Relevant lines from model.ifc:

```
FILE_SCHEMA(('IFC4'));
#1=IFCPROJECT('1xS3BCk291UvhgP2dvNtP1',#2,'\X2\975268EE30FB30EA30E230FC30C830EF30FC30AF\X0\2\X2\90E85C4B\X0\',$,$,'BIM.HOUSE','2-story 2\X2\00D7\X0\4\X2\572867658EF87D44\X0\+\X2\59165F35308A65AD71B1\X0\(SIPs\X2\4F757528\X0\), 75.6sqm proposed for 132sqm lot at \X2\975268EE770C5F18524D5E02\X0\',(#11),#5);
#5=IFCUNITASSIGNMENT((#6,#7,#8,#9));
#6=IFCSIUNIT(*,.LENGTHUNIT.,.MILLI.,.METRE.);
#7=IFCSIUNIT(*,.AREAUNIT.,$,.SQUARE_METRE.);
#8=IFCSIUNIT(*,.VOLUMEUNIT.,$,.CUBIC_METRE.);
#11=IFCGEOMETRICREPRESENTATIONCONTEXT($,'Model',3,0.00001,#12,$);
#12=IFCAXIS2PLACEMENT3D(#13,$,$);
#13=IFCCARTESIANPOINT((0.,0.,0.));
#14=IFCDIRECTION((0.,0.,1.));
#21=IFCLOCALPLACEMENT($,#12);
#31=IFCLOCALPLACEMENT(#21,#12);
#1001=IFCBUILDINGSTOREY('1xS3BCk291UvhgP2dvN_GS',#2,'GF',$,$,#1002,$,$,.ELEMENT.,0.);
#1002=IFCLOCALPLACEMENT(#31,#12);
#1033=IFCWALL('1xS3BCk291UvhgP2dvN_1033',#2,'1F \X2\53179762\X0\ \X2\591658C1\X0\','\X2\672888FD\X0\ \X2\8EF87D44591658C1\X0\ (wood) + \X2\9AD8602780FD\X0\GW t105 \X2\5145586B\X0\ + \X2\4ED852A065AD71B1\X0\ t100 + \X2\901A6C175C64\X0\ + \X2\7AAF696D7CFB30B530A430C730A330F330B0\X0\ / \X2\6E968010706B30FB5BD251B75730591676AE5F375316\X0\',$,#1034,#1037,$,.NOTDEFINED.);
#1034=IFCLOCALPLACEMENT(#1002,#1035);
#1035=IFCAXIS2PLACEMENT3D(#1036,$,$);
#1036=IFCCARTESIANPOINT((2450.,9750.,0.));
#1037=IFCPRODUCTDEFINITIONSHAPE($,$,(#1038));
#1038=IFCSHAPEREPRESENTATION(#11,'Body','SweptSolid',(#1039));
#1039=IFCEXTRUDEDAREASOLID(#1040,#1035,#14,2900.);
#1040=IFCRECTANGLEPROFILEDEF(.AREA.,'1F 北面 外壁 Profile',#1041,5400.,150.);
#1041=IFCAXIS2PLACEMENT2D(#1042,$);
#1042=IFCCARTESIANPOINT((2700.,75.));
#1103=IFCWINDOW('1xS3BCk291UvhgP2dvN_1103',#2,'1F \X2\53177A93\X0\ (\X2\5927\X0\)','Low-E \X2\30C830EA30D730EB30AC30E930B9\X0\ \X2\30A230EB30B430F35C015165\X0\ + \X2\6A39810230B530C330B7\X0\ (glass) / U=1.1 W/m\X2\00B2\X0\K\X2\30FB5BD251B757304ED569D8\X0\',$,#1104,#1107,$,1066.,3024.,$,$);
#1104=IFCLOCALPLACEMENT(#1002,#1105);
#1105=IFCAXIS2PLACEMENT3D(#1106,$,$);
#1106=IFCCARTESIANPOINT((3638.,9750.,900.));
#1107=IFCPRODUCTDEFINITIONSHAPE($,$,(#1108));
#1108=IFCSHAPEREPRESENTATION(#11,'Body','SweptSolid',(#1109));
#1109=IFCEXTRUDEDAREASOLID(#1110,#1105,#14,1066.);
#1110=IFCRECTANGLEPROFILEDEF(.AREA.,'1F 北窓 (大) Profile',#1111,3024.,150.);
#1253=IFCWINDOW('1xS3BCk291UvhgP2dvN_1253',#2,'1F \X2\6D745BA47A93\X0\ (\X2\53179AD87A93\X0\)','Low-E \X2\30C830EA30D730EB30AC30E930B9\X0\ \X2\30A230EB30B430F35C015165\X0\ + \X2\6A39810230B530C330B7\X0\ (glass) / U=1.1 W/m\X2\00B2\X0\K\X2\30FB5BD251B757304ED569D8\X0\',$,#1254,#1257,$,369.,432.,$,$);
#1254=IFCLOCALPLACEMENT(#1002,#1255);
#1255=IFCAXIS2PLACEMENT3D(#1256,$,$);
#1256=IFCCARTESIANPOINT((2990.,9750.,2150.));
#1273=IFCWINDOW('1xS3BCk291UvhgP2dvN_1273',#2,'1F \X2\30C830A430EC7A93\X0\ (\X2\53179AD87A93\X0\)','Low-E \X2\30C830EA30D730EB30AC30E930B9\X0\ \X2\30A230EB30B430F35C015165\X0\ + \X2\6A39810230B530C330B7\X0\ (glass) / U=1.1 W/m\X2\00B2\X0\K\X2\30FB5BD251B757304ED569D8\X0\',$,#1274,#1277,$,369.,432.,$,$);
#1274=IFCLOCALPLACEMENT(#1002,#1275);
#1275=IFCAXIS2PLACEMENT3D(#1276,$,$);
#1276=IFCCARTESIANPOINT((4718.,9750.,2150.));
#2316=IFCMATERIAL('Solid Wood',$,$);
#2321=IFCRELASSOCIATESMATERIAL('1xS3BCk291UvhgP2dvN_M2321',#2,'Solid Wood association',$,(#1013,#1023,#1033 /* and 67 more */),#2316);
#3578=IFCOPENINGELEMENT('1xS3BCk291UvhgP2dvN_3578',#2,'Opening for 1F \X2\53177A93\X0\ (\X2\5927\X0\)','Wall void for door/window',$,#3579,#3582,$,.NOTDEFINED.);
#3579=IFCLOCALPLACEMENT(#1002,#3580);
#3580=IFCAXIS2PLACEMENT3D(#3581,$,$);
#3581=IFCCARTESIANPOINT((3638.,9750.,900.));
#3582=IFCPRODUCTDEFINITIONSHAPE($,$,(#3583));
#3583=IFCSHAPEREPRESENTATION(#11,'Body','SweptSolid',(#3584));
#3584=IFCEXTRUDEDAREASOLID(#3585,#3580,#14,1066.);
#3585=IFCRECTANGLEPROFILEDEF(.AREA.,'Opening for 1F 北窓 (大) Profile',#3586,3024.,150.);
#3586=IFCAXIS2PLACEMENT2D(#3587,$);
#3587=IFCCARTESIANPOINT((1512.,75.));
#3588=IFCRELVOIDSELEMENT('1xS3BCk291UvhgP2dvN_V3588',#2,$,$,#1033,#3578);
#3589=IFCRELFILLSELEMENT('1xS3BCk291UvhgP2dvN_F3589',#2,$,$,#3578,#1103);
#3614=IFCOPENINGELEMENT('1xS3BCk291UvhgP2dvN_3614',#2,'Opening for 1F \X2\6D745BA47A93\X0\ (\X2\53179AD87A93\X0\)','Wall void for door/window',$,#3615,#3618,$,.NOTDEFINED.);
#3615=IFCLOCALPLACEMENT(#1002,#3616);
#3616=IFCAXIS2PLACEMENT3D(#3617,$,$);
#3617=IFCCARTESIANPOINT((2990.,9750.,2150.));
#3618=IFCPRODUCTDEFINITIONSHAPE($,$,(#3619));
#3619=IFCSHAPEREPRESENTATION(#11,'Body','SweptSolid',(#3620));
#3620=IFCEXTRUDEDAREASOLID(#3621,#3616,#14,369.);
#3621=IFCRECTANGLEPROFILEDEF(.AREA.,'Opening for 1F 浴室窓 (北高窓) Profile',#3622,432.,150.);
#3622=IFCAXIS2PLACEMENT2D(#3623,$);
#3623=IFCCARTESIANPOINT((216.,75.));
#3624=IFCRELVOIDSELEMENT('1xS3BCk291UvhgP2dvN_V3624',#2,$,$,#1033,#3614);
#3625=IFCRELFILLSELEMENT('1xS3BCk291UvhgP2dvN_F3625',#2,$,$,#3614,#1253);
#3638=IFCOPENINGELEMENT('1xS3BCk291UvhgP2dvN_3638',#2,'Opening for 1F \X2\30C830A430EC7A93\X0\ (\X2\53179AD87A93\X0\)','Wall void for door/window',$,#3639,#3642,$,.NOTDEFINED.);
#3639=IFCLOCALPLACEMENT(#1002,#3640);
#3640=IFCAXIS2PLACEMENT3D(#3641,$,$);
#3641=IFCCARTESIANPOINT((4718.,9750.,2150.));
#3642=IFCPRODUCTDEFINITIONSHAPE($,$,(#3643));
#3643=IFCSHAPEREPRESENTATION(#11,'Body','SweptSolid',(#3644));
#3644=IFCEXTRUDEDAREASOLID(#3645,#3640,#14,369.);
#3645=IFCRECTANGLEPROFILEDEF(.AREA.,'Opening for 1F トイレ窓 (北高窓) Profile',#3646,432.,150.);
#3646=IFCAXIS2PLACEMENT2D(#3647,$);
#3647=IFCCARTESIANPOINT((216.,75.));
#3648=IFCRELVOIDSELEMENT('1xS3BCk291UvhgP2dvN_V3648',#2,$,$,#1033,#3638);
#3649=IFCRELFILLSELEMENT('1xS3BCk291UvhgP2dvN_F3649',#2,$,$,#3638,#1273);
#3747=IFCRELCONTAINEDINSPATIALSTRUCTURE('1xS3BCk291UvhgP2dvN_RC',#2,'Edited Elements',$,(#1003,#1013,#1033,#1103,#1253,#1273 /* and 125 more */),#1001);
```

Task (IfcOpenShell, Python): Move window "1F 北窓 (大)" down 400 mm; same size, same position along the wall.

```python
import numpy as np
import ifcopenshell
import ifcopenshell.api.geometry
import ifcopenshell.util.placement
import ifcopenshell.util.unit

model = ifcopenshell.open("model.ifc")
unit_scale = ifcopenshell.util.unit.calculate_unit_scale(model)

window = model.by_guid("1xS3BCk291UvhgP2dvN_1103")
opening = window.FillsVoids[0].RelatingOpeningElement
dz = -0.4 / unit_scale

shift = np.array([0.0, 0.0, dz])
# The window is not placed relative to its opening, so move both.
for product in (opening, window):
    matrix = ifcopenshell.util.placement.get_local_placement(product.ObjectPlacement)
    matrix[:3, 3] += shift
    ifcopenshell.api.geometry.edit_object_placement(model, product=product, matrix=matrix, is_si=False)

print(f"moved by {dz * unit_scale:+.3f} m")

model.write("model-out.ifc")
```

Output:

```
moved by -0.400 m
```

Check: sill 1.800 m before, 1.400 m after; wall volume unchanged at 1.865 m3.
